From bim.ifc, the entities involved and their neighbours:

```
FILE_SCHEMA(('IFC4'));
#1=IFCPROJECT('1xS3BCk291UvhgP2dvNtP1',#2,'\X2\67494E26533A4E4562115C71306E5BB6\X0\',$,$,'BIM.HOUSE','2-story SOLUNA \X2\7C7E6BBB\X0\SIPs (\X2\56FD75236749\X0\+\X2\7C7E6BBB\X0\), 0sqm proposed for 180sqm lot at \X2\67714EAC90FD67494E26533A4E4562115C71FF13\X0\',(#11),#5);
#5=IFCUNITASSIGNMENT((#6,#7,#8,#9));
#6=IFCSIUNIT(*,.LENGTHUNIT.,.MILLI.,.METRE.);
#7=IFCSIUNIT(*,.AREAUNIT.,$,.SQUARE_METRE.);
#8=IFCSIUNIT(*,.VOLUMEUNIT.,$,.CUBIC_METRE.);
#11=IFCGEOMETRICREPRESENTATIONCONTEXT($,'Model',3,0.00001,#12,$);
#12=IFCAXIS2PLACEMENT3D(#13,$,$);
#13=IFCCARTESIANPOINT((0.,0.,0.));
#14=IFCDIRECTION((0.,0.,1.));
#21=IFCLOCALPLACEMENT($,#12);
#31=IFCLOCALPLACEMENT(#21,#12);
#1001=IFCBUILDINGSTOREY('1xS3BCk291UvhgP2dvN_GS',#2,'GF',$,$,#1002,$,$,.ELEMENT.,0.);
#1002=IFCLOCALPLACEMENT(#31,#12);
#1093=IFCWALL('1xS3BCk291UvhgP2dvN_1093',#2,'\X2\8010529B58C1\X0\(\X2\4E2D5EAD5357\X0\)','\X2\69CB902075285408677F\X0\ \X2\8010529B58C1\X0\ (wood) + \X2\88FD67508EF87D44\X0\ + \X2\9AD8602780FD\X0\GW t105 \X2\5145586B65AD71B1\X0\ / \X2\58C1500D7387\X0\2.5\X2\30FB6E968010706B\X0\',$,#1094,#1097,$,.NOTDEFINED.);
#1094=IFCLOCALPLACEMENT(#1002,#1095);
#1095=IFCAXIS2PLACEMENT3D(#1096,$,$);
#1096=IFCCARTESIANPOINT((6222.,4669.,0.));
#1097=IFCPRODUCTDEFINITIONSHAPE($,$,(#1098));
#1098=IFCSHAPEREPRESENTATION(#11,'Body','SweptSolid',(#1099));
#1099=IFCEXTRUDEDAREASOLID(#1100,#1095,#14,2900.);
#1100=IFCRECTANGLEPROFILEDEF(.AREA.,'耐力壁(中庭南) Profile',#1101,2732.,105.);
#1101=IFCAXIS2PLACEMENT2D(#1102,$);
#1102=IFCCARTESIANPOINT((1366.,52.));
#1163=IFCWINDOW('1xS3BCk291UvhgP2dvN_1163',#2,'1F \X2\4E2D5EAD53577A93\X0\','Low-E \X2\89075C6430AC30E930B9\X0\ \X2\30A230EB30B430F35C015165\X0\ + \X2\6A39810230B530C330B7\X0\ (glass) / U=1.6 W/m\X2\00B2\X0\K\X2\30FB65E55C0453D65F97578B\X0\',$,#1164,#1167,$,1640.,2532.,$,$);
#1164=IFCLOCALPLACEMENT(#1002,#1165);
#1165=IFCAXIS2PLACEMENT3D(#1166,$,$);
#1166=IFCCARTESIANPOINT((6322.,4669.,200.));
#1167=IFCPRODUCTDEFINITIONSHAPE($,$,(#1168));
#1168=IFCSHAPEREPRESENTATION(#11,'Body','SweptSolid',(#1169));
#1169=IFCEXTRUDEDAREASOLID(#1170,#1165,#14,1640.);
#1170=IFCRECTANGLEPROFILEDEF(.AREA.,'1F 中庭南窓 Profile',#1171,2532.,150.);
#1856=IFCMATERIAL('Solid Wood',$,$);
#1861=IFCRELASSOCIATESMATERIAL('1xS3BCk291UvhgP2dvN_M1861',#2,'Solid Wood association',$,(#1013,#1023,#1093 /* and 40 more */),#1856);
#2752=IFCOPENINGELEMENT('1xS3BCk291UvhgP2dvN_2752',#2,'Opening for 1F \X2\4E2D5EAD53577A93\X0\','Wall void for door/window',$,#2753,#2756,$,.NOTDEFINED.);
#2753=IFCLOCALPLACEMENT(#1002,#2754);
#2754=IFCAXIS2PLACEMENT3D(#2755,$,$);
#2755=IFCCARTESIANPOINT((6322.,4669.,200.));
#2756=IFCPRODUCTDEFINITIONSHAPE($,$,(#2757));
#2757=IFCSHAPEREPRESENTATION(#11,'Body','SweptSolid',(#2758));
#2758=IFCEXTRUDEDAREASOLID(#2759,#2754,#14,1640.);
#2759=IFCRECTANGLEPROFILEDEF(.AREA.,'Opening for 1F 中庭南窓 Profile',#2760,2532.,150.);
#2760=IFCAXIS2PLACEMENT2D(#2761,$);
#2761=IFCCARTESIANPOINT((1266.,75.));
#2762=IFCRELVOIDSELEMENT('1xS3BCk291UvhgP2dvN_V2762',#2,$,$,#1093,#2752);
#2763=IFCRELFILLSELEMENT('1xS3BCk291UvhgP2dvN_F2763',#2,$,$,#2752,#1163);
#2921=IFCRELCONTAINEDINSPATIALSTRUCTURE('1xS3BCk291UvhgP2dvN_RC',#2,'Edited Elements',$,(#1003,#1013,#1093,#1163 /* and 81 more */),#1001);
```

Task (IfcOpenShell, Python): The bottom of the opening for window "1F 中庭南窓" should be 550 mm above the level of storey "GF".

```python
import numpy as np
import ifcopenshell
import ifcopenshell.api.geometry
import ifcopenshell.geom
import ifcopenshell.util.element
import ifcopenshell.util.placement
import ifcopenshell.util.shape
import ifcopenshell.util.unit

model = ifcopenshell.open("bim.ifc")
unit_scale = ifcopenshell.util.unit.calculate_unit_scale(model)

window = model.by_id(1163)
opening = window.FillsVoids[0].RelatingOpeningElement
storey = ifcopenshell.util.element.get_container(window, ifc_class="IfcBuildingStorey")
level = ifcopenshell.util.placement.get_local_placement(storey.ObjectPlacement)[2, 3]

# The opening's origin need not be at the sill, so measure its lowest point.
shape = ifcopenshell.geom.create_shape(ifcopenshell.geom.settings(), opening)
bottom = ifcopenshell.util.shape.get_shape_bottom_elevation(shape, shape.geometry) / unit_scale
dz = level + 0.55 / unit_scale - bottom

shift = np.array([0.0, 0.0, dz])
# The window is not placed relative to its opening, so move both.
for product in (opening, window):
    matrix = ifcopenshell.util.placement.get_local_placement(product.ObjectPlacement)
    matrix[:3, 3] += shift
    ifcopenshell.api.geometry.edit_object_placement(model, product=product, matrix=matrix, is_si=False)

print(f"moved by {dz * unit_scale:+.3f} m")

model.write("bim_v2.ifc")
```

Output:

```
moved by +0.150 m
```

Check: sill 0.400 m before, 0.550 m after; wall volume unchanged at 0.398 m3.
